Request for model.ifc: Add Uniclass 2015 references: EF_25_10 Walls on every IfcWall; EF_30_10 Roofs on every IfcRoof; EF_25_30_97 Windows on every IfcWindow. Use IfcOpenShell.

First a look at what the model holds.

```python
import ifcopenshell

model = ifcopenshell.open("model.ifc")
print(model.schema)
print("classifications:", [c.Name for c in model.by_type("IfcClassification")])
for ifc_class in ("IfcDoor", "IfcRoof", "IfcStair", "IfcWall", "IfcWindow"):
    print(ifc_class, len(model.by_type(ifc_class)))
```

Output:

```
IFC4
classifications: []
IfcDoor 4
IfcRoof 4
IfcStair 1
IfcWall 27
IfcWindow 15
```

```python
import ifcopenshell
import ifcopenshell.api.classification

model = ifcopenshell.open("model.ifc")

system = ifcopenshell.api.classification.add_classification(model, classification="Uniclass 2015")

codes = {
    "IfcWall": ("EF_25_10", "Walls"),
    "IfcRoof": ("EF_30_10", "Roofs"),
    "IfcWindow": ("EF_25_30_97", "Windows"),
}
for ifc_class, (code, name) in codes.items():
    products = model.by_type(ifc_class)
    ifcopenshell.api.classification.add_reference(
        model, products=products, classification=system, identification=code, name=name
    )
    print(code, len(products))

model.write("model-out.ifc")
```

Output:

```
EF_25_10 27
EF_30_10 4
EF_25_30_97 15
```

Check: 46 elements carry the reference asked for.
